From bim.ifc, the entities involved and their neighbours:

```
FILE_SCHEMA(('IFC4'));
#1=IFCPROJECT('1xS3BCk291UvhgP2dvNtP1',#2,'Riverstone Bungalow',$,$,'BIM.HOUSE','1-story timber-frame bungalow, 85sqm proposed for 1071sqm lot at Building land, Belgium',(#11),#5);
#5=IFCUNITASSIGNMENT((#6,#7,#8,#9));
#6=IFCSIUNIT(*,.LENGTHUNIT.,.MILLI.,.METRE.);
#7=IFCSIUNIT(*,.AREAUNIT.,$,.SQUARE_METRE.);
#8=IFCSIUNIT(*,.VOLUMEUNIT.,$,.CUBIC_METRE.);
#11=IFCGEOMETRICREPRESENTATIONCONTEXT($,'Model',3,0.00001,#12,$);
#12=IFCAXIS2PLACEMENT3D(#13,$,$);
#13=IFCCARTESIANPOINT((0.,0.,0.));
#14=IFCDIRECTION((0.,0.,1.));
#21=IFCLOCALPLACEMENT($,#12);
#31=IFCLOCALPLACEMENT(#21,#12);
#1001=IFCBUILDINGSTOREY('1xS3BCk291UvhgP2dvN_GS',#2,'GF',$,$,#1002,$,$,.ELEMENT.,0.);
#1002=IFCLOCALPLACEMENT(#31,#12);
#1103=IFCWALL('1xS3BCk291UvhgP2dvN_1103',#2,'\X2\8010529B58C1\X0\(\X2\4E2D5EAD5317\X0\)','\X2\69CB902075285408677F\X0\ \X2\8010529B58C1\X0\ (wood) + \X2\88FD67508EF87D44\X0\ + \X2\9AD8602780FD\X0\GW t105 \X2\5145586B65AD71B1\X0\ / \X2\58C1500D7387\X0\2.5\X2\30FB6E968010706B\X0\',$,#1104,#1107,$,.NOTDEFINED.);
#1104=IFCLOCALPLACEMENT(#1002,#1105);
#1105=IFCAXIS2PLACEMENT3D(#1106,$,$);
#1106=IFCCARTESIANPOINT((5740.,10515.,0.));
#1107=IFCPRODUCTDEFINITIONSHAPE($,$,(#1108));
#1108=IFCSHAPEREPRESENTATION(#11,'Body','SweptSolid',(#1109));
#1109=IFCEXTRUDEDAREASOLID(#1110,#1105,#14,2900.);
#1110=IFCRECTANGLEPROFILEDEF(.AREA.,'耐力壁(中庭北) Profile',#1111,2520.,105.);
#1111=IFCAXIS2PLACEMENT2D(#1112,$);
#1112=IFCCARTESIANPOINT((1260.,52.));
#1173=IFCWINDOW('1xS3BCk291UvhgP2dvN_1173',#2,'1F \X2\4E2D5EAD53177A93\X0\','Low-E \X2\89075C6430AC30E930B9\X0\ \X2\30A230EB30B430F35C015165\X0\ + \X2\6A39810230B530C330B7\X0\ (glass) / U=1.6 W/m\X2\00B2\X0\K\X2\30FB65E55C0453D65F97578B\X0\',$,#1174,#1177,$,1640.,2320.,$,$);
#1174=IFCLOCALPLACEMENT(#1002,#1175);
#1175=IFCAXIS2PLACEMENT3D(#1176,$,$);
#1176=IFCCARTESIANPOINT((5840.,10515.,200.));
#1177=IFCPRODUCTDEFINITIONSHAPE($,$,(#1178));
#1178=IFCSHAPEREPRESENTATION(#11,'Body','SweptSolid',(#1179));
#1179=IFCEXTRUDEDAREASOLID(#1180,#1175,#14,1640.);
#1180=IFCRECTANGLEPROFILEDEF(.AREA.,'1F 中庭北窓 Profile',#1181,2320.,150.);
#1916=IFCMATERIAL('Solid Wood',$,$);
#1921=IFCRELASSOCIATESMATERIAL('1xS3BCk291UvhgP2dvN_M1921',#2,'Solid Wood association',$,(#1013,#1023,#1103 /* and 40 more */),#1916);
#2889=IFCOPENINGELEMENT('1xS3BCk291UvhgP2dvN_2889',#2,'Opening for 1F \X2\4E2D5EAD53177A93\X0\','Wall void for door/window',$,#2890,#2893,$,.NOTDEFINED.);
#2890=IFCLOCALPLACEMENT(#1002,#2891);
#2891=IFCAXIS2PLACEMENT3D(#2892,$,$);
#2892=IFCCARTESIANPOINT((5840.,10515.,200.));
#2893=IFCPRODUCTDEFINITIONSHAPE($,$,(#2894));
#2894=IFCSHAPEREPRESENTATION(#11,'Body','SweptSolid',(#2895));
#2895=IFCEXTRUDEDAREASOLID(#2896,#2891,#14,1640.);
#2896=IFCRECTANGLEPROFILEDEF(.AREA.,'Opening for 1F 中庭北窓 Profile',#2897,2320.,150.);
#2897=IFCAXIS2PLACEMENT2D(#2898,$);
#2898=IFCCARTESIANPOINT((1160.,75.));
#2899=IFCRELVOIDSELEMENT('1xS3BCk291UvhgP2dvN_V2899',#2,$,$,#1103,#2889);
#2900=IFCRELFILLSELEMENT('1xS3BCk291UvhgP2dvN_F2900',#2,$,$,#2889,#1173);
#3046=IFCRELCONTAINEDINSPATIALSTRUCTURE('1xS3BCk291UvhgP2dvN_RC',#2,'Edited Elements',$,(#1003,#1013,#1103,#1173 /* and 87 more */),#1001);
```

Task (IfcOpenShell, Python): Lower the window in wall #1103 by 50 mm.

```python
import numpy as np
import ifcopenshell
import ifcopenshell.api.geometry
import ifcopenshell.util.placement
import ifcopenshell.util.unit

model = ifcopenshell.open("bim.ifc")
unit_scale = ifcopenshell.util.unit.calculate_unit_scale(model)

window = model.by_guid("1xS3BCk291UvhgP2dvN_1173")
opening = window.FillsVoids[0].RelatingOpeningElement
dz = -0.05 / unit_scale

shift = np.array([0.0, 0.0, dz])
# The window is not placed relative to its opening, so move both.
for product in (opening, window):
    matrix = ifcopenshell.util.placement.get_local_placement(product.ObjectPlacement)
    matrix[:3, 3] += shift
    ifcopenshell.api.geometry.edit_object_placement(model, product=product, matrix=matrix, is_si=False)

print(f"moved by {dz * unit_scale:+.3f} m")

model.write("bim_edited.ifc")
```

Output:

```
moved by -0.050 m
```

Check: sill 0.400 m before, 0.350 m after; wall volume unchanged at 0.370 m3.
